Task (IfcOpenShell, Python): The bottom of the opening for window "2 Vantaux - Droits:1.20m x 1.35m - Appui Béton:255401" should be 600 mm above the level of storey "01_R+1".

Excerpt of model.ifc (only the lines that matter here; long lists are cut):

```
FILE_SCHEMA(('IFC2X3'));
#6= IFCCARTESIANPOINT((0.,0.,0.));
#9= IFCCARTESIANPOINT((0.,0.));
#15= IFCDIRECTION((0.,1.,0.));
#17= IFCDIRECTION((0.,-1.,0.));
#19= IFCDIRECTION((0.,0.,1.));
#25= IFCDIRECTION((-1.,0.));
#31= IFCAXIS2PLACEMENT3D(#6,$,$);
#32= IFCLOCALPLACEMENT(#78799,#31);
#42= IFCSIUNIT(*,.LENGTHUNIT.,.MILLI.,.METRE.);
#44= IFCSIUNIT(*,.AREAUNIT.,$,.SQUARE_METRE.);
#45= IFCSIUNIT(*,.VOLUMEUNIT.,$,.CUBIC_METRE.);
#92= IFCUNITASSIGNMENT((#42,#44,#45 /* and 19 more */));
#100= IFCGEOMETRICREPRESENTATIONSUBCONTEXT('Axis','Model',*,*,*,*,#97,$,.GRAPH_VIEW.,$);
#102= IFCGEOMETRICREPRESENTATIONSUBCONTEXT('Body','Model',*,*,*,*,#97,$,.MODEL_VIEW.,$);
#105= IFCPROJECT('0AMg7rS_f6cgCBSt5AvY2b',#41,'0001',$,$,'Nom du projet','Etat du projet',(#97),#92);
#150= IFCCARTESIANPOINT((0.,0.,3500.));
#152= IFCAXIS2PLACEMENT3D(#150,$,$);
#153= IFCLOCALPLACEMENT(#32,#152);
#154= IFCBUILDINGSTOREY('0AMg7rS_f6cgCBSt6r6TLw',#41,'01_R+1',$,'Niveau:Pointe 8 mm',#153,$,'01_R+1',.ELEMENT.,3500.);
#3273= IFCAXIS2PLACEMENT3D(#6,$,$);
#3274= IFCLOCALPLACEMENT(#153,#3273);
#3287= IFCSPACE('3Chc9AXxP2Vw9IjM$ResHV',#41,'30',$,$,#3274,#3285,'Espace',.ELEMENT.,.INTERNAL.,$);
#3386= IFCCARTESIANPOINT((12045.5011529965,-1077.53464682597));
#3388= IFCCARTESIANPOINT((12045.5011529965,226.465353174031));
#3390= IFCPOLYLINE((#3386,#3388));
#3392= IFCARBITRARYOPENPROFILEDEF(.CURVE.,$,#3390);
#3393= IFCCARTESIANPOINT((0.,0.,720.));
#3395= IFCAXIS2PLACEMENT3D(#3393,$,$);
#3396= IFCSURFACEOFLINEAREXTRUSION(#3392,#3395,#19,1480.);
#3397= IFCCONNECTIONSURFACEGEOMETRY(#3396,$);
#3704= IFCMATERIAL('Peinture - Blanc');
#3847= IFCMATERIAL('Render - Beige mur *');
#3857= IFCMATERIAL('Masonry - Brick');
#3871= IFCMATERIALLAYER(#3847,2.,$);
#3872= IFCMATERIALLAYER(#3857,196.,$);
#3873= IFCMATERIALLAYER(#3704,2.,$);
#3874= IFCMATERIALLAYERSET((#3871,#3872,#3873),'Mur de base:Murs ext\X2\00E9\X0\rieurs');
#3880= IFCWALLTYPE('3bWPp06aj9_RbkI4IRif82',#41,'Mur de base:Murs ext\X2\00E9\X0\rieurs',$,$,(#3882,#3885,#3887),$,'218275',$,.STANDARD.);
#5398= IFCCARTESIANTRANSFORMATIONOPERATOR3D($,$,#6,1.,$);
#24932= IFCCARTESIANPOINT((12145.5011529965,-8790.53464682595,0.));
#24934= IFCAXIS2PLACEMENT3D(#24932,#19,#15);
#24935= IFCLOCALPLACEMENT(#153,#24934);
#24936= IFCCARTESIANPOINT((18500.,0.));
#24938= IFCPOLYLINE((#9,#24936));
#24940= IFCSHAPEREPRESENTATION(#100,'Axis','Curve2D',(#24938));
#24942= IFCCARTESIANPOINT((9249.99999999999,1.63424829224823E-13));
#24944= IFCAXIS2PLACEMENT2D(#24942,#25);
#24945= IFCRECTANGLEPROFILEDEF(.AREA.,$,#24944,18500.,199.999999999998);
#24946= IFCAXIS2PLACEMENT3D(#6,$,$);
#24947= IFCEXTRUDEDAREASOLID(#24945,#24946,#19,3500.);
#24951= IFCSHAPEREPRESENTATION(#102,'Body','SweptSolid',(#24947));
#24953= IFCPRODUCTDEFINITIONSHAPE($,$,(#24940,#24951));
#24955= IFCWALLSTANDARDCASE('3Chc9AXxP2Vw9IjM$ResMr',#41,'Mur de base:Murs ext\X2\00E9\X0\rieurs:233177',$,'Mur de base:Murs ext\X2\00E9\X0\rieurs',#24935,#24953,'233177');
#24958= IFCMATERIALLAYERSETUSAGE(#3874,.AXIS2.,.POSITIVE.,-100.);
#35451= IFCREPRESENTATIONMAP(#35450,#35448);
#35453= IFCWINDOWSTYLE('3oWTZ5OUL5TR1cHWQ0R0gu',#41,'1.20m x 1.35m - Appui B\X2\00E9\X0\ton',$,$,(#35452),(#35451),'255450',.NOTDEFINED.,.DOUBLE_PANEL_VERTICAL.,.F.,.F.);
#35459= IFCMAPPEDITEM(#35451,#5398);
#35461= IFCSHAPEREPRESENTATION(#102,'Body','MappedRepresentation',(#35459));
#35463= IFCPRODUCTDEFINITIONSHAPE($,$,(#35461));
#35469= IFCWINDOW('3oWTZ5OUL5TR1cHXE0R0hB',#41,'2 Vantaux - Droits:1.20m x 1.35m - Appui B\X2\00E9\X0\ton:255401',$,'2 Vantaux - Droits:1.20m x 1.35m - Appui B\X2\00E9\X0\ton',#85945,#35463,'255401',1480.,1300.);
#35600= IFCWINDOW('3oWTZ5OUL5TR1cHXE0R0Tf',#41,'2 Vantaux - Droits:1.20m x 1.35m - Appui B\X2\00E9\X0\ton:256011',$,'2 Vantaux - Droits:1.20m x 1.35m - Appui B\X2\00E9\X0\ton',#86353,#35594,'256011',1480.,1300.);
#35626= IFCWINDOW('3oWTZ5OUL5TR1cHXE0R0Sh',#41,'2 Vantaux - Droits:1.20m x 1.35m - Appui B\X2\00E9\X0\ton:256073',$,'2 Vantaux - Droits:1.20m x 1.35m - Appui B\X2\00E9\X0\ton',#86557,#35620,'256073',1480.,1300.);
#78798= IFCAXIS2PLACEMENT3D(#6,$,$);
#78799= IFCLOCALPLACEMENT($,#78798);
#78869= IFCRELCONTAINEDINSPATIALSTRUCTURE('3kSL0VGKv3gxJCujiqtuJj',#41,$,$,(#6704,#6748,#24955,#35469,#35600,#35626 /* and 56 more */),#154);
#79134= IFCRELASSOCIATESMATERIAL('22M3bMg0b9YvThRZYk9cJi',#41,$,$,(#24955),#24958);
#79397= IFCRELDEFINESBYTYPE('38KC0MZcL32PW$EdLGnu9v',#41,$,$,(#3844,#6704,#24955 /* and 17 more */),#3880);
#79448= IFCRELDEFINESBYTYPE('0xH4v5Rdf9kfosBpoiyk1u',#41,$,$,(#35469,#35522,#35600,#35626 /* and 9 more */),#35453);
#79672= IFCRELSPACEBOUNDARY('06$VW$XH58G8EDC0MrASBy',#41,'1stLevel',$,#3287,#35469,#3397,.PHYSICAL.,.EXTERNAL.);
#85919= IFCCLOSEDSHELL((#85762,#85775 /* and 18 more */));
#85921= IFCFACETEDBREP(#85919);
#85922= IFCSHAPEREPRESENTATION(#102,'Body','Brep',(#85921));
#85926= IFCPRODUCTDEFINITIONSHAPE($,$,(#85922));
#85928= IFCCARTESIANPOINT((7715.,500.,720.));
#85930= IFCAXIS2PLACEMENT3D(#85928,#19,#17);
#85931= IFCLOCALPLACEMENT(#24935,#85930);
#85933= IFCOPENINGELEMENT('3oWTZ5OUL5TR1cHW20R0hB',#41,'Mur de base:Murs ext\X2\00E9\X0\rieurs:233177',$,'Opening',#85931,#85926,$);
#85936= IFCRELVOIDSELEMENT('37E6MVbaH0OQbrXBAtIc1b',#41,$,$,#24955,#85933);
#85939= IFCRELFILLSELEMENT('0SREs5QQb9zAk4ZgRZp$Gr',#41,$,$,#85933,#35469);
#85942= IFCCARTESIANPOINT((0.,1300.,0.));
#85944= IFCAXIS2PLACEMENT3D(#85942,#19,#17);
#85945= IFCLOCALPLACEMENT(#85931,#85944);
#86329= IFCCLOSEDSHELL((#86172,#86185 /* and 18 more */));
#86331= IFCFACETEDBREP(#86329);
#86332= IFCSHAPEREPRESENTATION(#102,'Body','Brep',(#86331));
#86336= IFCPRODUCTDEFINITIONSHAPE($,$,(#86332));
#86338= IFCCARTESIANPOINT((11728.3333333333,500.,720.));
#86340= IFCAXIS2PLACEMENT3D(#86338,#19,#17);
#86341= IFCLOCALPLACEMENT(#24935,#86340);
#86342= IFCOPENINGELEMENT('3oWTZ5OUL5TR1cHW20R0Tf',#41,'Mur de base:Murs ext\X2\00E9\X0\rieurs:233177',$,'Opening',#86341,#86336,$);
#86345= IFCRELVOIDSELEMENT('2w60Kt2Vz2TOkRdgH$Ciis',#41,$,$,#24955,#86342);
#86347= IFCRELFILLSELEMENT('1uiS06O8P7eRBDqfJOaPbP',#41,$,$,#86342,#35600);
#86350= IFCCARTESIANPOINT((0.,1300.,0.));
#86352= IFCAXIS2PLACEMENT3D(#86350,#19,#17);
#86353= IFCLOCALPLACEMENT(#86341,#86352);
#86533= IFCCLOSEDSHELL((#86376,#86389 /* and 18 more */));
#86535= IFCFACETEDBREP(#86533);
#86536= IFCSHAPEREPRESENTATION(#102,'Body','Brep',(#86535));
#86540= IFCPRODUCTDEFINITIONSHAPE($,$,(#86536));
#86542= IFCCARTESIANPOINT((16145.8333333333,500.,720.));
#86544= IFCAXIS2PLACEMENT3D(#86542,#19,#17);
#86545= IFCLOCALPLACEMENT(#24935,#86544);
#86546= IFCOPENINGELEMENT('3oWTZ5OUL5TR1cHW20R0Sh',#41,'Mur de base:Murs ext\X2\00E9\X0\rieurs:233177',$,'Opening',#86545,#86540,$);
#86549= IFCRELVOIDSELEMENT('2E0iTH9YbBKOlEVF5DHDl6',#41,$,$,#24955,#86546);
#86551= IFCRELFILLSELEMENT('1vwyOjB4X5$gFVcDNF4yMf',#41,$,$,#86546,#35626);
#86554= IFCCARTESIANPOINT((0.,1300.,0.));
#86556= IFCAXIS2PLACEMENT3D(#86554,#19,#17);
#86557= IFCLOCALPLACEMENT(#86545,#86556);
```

```python
import numpy as np
import ifcopenshell
import ifcopenshell.api.geometry
import ifcopenshell.geom
import ifcopenshell.util.element
import ifcopenshell.util.placement
import ifcopenshell.util.shape
import ifcopenshell.util.unit

model = ifcopenshell.open("model.ifc")
unit_scale = ifcopenshell.util.unit.calculate_unit_scale(model)

window = model.by_guid("3oWTZ5OUL5TR1cHXE0R0hB")
opening = window.FillsVoids[0].RelatingOpeningElement
storey = ifcopenshell.util.element.get_container(window, ifc_class="IfcBuildingStorey")
level = ifcopenshell.util.placement.get_local_placement(storey.ObjectPlacement)[2, 3]

# The opening's origin need not be at the sill, so measure its lowest point.
shape = ifcopenshell.geom.create_shape(ifcopenshell.geom.settings(), opening)
bottom = ifcopenshell.util.shape.get_shape_bottom_elevation(shape, shape.geometry) / unit_scale
dz = level + 600.0 - bottom

shift = np.array([0.0, 0.0, dz])
# The window is placed relative to its opening, so it follows when the opening moves.
matrix = ifcopenshell.util.placement.get_local_placement(opening.ObjectPlacement)
matrix[:3, 3] += shift
ifcopenshell.api.geometry.edit_object_placement(
    model, product=opening, matrix=matrix, is_si=False, should_transform_children=True
)

# Space boundary surfaces are stored in each space's coordinates; move them too.
for rel in window.ProvidesBoundaries:
    if not rel.ConnectionGeometry:
        continue
    surface = rel.ConnectionGeometry.SurfaceOnRelatingElement
    space_matrix = ifcopenshell.util.placement.get_local_placement(rel.RelatingSpace.ObjectPlacement)
    point = np.array(surface.Position.Location.Coordinates) + space_matrix[:3, :3].T @ shift
    surface.Position = model.createIfcAxis2Placement3D(
        model.createIfcCartesianPoint(point.tolist()), surface.Position.Axis, surface.Position.RefDirection
    )

print(f"moved by {dz * unit_scale:+.3f} m")

model.write("model_edited.ifc")
```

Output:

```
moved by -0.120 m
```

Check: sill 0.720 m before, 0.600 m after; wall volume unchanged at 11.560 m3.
